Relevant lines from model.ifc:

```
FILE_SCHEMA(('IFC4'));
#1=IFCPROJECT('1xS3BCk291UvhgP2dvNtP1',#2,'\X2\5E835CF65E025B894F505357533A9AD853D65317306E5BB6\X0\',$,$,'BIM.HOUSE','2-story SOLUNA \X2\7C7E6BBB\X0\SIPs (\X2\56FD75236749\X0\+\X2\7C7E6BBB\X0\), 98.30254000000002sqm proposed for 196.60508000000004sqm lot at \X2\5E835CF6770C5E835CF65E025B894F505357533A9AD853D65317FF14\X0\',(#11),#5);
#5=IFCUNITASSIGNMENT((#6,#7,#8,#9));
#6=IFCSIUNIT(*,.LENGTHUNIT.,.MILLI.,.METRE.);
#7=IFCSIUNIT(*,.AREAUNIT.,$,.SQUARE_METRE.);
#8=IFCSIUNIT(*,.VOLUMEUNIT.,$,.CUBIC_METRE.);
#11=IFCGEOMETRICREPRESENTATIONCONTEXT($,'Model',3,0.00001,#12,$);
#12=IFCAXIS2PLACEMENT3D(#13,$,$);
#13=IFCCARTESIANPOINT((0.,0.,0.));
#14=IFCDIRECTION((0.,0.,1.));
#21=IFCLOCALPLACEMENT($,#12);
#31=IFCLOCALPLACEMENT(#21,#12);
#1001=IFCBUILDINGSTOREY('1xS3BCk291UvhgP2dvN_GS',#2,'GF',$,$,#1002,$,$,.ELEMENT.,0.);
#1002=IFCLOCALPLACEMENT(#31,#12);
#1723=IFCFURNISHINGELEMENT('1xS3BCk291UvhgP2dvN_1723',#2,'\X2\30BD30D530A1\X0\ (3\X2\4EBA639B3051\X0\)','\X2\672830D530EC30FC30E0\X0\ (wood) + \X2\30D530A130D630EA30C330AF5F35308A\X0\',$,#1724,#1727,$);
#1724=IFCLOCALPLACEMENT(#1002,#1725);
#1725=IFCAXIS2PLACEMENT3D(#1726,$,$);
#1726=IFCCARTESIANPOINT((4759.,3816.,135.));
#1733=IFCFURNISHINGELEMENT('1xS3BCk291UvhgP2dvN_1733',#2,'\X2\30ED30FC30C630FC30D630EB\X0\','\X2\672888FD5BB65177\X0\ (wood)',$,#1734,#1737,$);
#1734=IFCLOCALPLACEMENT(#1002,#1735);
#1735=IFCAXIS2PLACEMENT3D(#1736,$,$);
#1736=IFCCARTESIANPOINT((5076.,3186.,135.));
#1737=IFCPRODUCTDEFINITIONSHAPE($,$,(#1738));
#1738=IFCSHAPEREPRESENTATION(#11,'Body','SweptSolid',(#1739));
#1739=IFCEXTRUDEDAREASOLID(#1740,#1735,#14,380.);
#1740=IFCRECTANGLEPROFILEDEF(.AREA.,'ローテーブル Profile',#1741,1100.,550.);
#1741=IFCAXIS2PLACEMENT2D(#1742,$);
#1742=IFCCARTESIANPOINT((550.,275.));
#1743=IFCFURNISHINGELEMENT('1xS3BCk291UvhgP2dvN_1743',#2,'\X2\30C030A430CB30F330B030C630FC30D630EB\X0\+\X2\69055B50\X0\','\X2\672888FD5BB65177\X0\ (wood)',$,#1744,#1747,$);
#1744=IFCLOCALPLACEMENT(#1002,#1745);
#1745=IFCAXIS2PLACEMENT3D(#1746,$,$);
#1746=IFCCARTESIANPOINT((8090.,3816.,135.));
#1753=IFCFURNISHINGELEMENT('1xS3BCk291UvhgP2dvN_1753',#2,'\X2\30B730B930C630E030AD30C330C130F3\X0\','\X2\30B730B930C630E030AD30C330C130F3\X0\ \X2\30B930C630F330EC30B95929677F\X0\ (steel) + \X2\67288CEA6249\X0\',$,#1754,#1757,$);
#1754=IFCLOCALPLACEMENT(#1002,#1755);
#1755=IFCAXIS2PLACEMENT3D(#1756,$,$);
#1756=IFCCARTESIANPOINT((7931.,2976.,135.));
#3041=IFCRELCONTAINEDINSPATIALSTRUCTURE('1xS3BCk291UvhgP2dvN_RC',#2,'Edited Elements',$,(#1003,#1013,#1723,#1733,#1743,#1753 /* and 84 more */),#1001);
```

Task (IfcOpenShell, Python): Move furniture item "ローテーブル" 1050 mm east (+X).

```python
import ifcopenshell
import ifcopenshell.api.geometry
import ifcopenshell.util.placement
import ifcopenshell.util.unit

model = ifcopenshell.open("model.ifc")
unit_scale = ifcopenshell.util.unit.calculate_unit_scale(model)

item = model.by_guid("1xS3BCk291UvhgP2dvN_1733")
matrix = ifcopenshell.util.placement.get_local_placement(item.ObjectPlacement)
matrix[0, 3] += 1.05 / unit_scale
ifcopenshell.api.geometry.edit_object_placement(model, product=item, matrix=matrix, is_si=False)

print(ifcopenshell.util.placement.get_local_placement(item.ObjectPlacement).round(3) + 0.0)

model.write("model_v2.ifc")
```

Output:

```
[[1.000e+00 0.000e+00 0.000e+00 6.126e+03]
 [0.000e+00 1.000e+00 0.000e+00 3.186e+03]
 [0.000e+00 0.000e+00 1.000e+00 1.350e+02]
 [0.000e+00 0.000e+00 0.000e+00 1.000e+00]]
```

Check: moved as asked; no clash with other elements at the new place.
